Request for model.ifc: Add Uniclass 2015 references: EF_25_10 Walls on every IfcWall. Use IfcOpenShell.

First a look at what the model holds.

```python
import ifcopenshell

model = ifcopenshell.open("model.ifc")
print(model.schema)
print("classifications:", [c.Name for c in model.by_type("IfcClassification")])
for ifc_class in ("IfcDoor", "IfcRoof", "IfcStair", "IfcWall", "IfcWindow"):
    print(ifc_class, len(model.by_type(ifc_class)))
```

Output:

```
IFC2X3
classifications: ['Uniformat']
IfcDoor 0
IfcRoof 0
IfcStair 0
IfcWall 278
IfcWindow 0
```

```python
import ifcopenshell
import ifcopenshell.api.classification

model = ifcopenshell.open("model.ifc")

# IFC2X3 requires Source and Edition and has no link from the project to the system.
system = model.create_entity("IfcClassification", Source="NBS", Edition="2015", Name="Uniclass 2015")

codes = {
    "IfcWall": ("EF_25_10", "Walls"),
}
for ifc_class, (code, name) in codes.items():
    products = model.by_type(ifc_class)
    ifcopenshell.api.classification.add_reference(
        model, products=products, classification=system, identification=code, name=name
    )
    print(code, len(products))

model.write("model_rev.ifc")
```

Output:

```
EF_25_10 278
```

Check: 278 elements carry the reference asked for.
